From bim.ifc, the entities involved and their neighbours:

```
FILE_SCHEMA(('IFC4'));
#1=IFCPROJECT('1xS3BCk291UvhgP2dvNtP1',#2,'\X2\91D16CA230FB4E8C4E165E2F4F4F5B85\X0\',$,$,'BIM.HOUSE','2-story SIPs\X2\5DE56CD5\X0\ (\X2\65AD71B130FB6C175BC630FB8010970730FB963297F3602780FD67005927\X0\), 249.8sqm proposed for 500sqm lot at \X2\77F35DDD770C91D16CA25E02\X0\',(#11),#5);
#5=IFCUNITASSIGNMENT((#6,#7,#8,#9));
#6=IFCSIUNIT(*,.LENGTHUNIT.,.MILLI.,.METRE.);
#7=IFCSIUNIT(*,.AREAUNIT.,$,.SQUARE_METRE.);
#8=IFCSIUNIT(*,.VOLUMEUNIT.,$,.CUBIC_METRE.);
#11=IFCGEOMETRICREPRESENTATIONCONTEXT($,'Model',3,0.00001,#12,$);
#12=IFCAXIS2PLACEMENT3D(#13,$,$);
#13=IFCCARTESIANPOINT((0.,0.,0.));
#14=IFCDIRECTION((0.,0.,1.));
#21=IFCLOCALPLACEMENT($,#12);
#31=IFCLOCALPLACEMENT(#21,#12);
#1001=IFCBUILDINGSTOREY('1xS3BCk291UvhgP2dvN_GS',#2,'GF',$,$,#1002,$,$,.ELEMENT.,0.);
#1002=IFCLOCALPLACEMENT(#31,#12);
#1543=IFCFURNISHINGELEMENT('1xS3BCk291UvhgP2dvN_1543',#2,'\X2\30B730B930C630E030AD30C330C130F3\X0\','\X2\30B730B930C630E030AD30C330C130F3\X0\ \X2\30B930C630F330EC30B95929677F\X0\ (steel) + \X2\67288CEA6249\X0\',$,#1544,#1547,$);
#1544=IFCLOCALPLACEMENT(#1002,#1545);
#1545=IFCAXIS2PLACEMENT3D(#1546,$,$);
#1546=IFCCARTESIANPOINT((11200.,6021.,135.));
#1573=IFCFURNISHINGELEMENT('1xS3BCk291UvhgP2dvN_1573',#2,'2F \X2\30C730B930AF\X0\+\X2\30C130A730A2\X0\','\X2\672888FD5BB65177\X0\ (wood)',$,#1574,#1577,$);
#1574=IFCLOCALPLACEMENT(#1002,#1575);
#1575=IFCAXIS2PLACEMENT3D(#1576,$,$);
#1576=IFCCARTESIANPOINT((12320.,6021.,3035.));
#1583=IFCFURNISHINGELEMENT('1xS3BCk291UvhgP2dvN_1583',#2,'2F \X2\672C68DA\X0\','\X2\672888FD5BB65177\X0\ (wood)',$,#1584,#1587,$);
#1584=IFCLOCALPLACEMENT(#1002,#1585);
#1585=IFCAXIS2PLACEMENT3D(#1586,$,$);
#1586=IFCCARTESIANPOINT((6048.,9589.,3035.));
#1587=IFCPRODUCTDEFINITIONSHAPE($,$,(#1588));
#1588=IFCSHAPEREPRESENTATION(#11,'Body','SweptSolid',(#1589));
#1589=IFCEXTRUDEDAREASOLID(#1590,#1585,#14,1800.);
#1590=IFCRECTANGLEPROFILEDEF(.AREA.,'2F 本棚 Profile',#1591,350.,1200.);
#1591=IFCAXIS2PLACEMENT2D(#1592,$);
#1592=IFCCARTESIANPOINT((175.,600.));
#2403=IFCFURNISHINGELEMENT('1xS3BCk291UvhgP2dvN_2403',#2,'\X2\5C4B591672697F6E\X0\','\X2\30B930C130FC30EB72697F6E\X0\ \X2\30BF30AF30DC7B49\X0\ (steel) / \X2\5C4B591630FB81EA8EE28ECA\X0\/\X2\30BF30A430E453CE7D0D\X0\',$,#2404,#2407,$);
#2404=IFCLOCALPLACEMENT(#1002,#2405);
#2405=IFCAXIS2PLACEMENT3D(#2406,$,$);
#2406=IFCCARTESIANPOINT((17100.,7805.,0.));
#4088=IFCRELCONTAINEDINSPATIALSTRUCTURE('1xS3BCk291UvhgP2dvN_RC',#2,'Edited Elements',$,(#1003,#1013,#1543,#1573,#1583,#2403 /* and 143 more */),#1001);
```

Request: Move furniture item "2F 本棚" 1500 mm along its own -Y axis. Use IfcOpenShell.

```python
import ifcopenshell
import ifcopenshell.api.geometry
import ifcopenshell.util.placement
import ifcopenshell.util.unit

model = ifcopenshell.open("bim.ifc")
unit_scale = ifcopenshell.util.unit.calculate_unit_scale(model)

item = model.by_guid("1xS3BCk291UvhgP2dvN_1583")
matrix = ifcopenshell.util.placement.get_local_placement(item.ObjectPlacement)
matrix[:3, 3] -= matrix[:3, 1] * 1.5 / unit_scale
ifcopenshell.api.geometry.edit_object_placement(model, product=item, matrix=matrix, is_si=False)

print(ifcopenshell.util.placement.get_local_placement(item.ObjectPlacement).round(3) + 0.0)

model.write("bim_rev.ifc")
```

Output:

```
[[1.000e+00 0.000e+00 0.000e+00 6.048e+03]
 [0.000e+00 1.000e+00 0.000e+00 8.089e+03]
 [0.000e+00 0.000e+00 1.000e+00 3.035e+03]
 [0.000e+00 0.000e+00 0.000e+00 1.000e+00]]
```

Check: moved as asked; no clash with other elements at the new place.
